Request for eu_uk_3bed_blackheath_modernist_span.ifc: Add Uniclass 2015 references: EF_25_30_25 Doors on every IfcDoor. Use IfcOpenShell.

First a look at what the model holds.

```python
import ifcopenshell

model = ifcopenshell.open("eu_uk_3bed_blackheath_modernist_span.ifc")
print(model.schema)
print("classifications:", [c.Name for c in model.by_type("IfcClassification")])
for ifc_class in ("IfcDoor", "IfcRoof", "IfcStair", "IfcWall", "IfcWindow"):
    print(ifc_class, len(model.by_type(ifc_class)))
```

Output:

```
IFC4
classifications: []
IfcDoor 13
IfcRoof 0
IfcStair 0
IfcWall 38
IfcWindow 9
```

```python
import ifcopenshell
import ifcopenshell.api.classification

model = ifcopenshell.open("eu_uk_3bed_blackheath_modernist_span.ifc")

system = ifcopenshell.api.classification.add_classification(model, classification="Uniclass 2015")

codes = {
    "IfcDoor": ("EF_25_30_25", "Doors"),
}
for ifc_class, (code, name) in codes.items():
    products = model.by_type(ifc_class)
    ifcopenshell.api.classification.add_reference(
        model, products=products, classification=system, identification=code, name=name
    )
    print(code, len(products))

model.write("eu_uk_3bed_blackheath_modernist_span-out.ifc")
```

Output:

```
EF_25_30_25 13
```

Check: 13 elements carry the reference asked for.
